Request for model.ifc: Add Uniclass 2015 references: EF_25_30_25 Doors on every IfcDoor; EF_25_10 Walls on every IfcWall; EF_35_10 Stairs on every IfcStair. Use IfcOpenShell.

First a look at what the model holds.

```python
import ifcopenshell

model = ifcopenshell.open("model.ifc")
print(model.schema)
print("classifications:", [c.Name for c in model.by_type("IfcClassification")])
for ifc_class in ("IfcDoor", "IfcRoof", "IfcStair", "IfcWall", "IfcWindow"):
    print(ifc_class, len(model.by_type(ifc_class)))
```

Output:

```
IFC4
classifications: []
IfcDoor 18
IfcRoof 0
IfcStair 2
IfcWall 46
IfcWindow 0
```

```python
import ifcopenshell
import ifcopenshell.api.classification

model = ifcopenshell.open("model.ifc")

system = ifcopenshell.api.classification.add_classification(model, classification="Uniclass 2015")

codes = {
    "IfcDoor": ("EF_25_30_25", "Doors"),
    "IfcWall": ("EF_25_10", "Walls"),
    "IfcStair": ("EF_35_10", "Stairs"),
}
for ifc_class, (code, name) in codes.items():
    products = model.by_type(ifc_class)
    ifcopenshell.api.classification.add_reference(
        model, products=products, classification=system, identification=code, name=name
    )
    print(code, len(products))

model.write("model_updated.ifc")
```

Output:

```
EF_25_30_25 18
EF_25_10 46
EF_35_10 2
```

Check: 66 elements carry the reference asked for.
